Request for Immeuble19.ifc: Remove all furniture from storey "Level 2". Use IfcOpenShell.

First a look at what the model holds.

```python
import ifcopenshell
import ifcopenshell.util.element

model = ifcopenshell.open("Immeuble19.ifc")
print(model.schema)
storey = next(s for s in model.by_type("IfcBuildingStorey") if s.Name == "Level 2")
furniture = [e for e in ifcopenshell.util.element.get_decomposition(storey) if e.is_a("IfcFurnishingElement")]
seen = {}
for e in furniture:
    element_type = ifcopenshell.util.element.get_type(e)
    name = element_type.Name if element_type not in (None, e) else None
    seen[name] = seen.get(name, 0) + 1
for name, count in sorted(seen.items(), key=str):
    print(count, "x", name)
```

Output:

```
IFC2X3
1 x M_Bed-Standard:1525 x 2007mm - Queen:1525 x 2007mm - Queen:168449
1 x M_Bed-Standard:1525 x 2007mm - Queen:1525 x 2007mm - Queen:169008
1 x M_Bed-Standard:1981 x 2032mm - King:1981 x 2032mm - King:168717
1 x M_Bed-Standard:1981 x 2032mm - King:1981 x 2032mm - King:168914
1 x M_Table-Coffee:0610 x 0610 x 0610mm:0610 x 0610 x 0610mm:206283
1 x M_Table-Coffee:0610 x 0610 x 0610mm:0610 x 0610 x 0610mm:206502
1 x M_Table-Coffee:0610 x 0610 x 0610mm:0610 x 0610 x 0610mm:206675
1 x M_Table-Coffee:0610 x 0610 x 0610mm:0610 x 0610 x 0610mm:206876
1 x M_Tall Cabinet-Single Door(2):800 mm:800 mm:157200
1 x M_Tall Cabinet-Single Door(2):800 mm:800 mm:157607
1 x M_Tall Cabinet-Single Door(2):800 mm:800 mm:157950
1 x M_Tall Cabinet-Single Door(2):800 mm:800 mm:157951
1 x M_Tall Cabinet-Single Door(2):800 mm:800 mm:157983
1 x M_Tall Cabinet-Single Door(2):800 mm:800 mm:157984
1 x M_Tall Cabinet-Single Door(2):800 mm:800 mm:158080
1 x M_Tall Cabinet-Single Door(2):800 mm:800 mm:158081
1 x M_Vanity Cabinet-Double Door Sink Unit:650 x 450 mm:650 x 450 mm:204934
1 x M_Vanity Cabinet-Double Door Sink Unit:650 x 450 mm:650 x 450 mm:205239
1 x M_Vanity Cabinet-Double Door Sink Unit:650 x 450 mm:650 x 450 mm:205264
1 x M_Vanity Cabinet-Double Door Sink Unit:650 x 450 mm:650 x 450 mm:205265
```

```python
import ifcopenshell
import ifcopenshell.api.root
import ifcopenshell.util.element

model = ifcopenshell.open("Immeuble19.ifc")

storey = next(s for s in model.by_type("IfcBuildingStorey") if s.Name == "Level 2")
furniture = [e for e in ifcopenshell.util.element.get_decomposition(storey) if e.is_a("IfcFurnishingElement")]

for e in furniture:
    ifcopenshell.api.root.remove_product(model, product=e)
print(len(furniture), "removed")

model.write("Immeuble19_v2.ifc")
```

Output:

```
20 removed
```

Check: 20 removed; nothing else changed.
